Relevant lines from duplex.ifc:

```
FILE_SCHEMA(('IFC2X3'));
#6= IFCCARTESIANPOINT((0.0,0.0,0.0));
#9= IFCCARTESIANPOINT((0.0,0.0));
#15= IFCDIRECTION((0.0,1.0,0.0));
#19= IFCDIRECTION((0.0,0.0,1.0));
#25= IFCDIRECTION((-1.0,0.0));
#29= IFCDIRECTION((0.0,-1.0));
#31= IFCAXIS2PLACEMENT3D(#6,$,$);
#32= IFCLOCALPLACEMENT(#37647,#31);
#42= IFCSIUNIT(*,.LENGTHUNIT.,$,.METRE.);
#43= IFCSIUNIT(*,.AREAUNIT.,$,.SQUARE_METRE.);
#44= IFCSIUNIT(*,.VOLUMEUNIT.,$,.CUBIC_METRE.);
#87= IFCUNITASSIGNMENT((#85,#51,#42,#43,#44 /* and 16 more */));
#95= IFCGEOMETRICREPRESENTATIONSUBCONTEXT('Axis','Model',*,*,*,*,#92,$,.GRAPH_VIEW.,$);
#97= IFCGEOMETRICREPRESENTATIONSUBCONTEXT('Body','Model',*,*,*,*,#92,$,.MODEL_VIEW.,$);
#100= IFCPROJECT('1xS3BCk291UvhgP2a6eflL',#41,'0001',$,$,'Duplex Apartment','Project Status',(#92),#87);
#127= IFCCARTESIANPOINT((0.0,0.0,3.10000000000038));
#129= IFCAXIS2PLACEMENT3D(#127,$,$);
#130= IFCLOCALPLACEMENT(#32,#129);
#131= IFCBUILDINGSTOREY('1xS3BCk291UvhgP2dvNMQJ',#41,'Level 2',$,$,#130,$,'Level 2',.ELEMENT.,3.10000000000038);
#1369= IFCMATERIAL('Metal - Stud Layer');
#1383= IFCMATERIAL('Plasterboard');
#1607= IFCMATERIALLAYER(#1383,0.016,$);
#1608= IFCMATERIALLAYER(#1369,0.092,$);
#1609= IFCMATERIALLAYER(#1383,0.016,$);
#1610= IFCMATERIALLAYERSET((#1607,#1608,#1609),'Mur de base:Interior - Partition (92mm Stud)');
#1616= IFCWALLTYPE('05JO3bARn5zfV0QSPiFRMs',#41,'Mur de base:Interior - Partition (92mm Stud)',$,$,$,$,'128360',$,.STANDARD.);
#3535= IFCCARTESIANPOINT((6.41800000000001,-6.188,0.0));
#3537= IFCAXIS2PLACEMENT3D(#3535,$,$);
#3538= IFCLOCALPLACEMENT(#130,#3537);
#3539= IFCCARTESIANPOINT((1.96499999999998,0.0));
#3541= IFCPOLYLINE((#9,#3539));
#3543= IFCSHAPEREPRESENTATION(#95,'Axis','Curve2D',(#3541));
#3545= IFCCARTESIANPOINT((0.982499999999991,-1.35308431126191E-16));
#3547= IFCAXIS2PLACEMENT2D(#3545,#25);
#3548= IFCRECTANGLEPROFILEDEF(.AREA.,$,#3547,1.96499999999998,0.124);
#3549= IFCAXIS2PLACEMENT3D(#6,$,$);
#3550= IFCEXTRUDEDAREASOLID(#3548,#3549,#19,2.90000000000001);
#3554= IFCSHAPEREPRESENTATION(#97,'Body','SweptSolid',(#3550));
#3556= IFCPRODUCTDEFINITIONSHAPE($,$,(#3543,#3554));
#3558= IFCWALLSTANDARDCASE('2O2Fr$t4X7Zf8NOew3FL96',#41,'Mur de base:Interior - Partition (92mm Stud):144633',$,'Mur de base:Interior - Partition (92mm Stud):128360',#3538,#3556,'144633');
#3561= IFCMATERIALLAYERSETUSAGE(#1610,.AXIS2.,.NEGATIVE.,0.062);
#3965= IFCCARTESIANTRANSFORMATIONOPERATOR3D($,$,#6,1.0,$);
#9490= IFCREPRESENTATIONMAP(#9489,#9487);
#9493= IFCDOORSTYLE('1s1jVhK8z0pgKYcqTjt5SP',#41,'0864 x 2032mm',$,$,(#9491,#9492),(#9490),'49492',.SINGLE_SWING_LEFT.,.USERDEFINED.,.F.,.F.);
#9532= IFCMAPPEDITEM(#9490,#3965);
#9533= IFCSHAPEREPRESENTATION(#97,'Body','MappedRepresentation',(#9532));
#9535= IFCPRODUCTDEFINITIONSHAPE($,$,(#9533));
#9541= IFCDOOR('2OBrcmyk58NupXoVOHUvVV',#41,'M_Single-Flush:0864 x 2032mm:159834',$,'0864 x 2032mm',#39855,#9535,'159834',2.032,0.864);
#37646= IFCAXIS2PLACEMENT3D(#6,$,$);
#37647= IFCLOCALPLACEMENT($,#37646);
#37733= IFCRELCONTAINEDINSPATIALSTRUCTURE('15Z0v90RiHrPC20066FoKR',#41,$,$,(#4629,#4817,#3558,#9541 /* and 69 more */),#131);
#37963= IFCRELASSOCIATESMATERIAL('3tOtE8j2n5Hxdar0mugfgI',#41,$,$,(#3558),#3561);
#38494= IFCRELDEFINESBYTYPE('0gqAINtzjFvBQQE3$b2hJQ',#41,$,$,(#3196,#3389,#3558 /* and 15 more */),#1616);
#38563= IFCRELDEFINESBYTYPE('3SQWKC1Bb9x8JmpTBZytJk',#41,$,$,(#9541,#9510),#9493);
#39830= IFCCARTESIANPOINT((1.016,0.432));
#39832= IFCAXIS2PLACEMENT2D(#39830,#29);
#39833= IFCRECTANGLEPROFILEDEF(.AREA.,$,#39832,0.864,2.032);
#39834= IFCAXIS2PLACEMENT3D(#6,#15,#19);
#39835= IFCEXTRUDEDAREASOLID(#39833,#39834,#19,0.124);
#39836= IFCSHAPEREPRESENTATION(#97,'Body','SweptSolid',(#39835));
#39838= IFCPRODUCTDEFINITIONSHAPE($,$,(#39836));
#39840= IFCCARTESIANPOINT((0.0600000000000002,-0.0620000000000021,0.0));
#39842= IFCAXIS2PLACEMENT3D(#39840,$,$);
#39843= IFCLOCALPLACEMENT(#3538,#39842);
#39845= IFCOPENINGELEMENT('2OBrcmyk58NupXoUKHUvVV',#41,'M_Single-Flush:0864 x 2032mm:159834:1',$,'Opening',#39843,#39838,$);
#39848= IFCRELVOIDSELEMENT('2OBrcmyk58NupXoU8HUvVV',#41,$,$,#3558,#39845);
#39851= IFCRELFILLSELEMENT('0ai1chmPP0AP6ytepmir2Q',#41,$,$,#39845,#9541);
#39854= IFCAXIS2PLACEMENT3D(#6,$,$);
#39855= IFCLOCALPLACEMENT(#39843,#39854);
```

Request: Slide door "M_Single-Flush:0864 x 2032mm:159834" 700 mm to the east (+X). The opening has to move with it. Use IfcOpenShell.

```python
import ifcopenshell
import ifcopenshell.api.geometry
import ifcopenshell.util.placement
import ifcopenshell.util.unit

model = ifcopenshell.open("duplex.ifc")
unit_scale = ifcopenshell.util.unit.calculate_unit_scale(model)

door = model.by_guid("2OBrcmyk58NupXoVOHUvVV")
opening = door.FillsVoids[0].RelatingOpeningElement
wall = opening.VoidsElements[0].RelatingBuildingElement

wall_matrix = ifcopenshell.util.placement.get_local_placement(wall.ObjectPlacement)
shift = wall_matrix[:3, 0] * 0.7 / unit_scale
before = ifcopenshell.util.placement.get_local_placement(door.ObjectPlacement)[:3, 3].copy()

# The door is placed relative to its opening, so it follows when the opening moves.
matrix = ifcopenshell.util.placement.get_local_placement(opening.ObjectPlacement)
matrix[:3, 3] += shift
ifcopenshell.api.geometry.edit_object_placement(
    model, product=opening, matrix=matrix, is_si=False, should_transform_children=True
)

after = ifcopenshell.util.placement.get_local_placement(door.ObjectPlacement)[:3, 3]
print("door moved by", (after - before).round(3) + 0.0)

model.write("duplex_updated.ifc")
```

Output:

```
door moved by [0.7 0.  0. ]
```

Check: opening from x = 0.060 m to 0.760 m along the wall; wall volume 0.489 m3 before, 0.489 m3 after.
